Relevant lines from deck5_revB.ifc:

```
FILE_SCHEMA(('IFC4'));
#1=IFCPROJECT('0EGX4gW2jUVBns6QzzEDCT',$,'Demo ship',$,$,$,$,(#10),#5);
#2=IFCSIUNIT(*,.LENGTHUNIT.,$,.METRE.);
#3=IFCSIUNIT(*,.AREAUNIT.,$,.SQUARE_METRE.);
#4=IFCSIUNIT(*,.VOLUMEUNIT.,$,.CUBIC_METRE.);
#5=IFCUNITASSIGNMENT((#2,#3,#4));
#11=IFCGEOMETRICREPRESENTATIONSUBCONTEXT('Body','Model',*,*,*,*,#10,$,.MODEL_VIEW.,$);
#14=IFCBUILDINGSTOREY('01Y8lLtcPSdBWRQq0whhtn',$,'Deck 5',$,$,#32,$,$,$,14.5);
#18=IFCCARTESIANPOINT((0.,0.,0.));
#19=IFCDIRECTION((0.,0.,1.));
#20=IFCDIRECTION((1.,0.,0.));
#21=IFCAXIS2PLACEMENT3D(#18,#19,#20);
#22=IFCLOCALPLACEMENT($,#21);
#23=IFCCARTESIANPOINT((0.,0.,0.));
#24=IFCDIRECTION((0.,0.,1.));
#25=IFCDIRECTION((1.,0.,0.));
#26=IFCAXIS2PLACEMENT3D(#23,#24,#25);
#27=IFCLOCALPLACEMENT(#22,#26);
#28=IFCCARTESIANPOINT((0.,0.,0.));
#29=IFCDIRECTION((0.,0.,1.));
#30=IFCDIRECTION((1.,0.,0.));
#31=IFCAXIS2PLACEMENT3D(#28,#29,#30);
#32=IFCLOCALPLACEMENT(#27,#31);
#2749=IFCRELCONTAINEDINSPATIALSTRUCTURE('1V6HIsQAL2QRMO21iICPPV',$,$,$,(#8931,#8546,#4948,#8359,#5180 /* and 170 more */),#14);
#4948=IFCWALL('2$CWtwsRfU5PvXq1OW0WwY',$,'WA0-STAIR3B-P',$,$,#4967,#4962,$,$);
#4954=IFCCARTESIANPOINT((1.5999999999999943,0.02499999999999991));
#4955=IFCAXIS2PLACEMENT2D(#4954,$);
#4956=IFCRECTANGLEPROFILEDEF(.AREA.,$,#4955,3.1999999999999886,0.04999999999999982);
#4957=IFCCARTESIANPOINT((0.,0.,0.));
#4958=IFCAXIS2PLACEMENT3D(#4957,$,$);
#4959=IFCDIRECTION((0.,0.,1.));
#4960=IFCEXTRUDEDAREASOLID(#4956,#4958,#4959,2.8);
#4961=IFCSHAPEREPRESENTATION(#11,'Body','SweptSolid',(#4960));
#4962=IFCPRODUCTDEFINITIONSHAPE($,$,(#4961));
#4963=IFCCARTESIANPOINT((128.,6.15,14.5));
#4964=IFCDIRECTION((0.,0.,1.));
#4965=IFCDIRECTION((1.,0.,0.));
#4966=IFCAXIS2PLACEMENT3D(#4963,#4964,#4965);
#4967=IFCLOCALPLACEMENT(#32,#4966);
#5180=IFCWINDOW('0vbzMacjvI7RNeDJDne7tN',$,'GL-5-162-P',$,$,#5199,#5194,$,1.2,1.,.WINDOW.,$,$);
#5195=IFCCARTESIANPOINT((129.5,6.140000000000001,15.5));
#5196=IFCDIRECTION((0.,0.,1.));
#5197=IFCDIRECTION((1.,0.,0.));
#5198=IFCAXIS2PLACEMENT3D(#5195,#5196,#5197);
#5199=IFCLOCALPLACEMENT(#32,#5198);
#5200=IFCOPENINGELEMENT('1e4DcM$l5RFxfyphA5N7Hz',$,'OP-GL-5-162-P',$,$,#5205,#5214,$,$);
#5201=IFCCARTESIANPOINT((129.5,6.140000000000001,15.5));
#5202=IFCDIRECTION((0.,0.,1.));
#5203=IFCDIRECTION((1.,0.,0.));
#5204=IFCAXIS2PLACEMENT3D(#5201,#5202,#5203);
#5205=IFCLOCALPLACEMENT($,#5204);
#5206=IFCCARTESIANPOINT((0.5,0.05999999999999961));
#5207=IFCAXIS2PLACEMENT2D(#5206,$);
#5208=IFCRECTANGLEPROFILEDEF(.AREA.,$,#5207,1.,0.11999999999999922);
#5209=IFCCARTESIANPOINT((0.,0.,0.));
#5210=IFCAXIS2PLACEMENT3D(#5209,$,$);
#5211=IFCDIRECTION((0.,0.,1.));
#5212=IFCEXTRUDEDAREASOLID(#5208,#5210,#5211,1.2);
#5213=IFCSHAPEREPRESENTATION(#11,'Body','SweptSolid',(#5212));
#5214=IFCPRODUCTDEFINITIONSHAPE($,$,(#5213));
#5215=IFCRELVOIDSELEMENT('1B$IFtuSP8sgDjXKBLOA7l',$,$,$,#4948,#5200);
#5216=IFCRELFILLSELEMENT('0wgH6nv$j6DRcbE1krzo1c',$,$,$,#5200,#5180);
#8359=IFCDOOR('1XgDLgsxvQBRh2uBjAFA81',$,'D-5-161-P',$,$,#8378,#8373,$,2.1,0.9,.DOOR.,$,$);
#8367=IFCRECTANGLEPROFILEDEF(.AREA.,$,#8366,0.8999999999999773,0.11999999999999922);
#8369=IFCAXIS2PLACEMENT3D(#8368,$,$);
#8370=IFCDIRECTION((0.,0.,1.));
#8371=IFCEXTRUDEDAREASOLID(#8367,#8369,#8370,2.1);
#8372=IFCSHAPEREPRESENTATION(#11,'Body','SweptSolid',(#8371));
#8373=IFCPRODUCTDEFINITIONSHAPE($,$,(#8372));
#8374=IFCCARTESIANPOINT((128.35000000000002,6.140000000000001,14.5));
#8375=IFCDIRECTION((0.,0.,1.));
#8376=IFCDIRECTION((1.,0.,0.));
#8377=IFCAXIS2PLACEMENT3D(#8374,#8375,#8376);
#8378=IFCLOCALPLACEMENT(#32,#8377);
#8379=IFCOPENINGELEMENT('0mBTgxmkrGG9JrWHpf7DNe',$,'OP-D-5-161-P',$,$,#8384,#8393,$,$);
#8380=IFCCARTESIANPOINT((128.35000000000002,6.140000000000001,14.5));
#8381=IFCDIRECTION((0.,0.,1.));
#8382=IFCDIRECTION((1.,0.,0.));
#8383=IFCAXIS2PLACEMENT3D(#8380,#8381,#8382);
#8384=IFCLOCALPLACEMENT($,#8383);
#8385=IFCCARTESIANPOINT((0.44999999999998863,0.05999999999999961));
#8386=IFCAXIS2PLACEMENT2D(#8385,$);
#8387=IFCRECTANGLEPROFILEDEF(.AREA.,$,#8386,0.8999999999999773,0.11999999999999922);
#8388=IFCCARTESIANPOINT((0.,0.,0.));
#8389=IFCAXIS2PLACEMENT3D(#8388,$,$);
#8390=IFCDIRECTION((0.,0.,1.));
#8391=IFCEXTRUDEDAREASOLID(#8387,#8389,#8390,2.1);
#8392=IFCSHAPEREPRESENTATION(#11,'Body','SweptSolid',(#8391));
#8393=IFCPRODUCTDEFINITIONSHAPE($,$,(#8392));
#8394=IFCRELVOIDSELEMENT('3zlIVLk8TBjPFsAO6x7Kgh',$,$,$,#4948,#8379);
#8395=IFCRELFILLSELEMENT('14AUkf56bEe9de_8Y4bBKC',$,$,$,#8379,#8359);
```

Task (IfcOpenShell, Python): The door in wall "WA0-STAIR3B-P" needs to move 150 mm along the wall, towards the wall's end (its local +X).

```python
import ifcopenshell
import ifcopenshell.api.geometry
import ifcopenshell.util.placement

model = ifcopenshell.open("deck5_revB.ifc")

door = model.by_id(8359)
opening = door.FillsVoids[0].RelatingOpeningElement
wall = opening.VoidsElements[0].RelatingBuildingElement

wall_matrix = ifcopenshell.util.placement.get_local_placement(wall.ObjectPlacement)
shift = wall_matrix[:3, 0] * 0.15
before = ifcopenshell.util.placement.get_local_placement(door.ObjectPlacement)[:3, 3].copy()

# The door is not placed relative to its opening, so move both.
for product in (opening, door):
    matrix = ifcopenshell.util.placement.get_local_placement(product.ObjectPlacement)
    matrix[:3, 3] += shift
    ifcopenshell.api.geometry.edit_object_placement(model, product=product, matrix=matrix, is_si=False)

after = ifcopenshell.util.placement.get_local_placement(door.ObjectPlacement)[:3, 3]
print("door moved by", (after - before).round(3) + 0.0)

model.write("deck5_revB-out.ifc")
```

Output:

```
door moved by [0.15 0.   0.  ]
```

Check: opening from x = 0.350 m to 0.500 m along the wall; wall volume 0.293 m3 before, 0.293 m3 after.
